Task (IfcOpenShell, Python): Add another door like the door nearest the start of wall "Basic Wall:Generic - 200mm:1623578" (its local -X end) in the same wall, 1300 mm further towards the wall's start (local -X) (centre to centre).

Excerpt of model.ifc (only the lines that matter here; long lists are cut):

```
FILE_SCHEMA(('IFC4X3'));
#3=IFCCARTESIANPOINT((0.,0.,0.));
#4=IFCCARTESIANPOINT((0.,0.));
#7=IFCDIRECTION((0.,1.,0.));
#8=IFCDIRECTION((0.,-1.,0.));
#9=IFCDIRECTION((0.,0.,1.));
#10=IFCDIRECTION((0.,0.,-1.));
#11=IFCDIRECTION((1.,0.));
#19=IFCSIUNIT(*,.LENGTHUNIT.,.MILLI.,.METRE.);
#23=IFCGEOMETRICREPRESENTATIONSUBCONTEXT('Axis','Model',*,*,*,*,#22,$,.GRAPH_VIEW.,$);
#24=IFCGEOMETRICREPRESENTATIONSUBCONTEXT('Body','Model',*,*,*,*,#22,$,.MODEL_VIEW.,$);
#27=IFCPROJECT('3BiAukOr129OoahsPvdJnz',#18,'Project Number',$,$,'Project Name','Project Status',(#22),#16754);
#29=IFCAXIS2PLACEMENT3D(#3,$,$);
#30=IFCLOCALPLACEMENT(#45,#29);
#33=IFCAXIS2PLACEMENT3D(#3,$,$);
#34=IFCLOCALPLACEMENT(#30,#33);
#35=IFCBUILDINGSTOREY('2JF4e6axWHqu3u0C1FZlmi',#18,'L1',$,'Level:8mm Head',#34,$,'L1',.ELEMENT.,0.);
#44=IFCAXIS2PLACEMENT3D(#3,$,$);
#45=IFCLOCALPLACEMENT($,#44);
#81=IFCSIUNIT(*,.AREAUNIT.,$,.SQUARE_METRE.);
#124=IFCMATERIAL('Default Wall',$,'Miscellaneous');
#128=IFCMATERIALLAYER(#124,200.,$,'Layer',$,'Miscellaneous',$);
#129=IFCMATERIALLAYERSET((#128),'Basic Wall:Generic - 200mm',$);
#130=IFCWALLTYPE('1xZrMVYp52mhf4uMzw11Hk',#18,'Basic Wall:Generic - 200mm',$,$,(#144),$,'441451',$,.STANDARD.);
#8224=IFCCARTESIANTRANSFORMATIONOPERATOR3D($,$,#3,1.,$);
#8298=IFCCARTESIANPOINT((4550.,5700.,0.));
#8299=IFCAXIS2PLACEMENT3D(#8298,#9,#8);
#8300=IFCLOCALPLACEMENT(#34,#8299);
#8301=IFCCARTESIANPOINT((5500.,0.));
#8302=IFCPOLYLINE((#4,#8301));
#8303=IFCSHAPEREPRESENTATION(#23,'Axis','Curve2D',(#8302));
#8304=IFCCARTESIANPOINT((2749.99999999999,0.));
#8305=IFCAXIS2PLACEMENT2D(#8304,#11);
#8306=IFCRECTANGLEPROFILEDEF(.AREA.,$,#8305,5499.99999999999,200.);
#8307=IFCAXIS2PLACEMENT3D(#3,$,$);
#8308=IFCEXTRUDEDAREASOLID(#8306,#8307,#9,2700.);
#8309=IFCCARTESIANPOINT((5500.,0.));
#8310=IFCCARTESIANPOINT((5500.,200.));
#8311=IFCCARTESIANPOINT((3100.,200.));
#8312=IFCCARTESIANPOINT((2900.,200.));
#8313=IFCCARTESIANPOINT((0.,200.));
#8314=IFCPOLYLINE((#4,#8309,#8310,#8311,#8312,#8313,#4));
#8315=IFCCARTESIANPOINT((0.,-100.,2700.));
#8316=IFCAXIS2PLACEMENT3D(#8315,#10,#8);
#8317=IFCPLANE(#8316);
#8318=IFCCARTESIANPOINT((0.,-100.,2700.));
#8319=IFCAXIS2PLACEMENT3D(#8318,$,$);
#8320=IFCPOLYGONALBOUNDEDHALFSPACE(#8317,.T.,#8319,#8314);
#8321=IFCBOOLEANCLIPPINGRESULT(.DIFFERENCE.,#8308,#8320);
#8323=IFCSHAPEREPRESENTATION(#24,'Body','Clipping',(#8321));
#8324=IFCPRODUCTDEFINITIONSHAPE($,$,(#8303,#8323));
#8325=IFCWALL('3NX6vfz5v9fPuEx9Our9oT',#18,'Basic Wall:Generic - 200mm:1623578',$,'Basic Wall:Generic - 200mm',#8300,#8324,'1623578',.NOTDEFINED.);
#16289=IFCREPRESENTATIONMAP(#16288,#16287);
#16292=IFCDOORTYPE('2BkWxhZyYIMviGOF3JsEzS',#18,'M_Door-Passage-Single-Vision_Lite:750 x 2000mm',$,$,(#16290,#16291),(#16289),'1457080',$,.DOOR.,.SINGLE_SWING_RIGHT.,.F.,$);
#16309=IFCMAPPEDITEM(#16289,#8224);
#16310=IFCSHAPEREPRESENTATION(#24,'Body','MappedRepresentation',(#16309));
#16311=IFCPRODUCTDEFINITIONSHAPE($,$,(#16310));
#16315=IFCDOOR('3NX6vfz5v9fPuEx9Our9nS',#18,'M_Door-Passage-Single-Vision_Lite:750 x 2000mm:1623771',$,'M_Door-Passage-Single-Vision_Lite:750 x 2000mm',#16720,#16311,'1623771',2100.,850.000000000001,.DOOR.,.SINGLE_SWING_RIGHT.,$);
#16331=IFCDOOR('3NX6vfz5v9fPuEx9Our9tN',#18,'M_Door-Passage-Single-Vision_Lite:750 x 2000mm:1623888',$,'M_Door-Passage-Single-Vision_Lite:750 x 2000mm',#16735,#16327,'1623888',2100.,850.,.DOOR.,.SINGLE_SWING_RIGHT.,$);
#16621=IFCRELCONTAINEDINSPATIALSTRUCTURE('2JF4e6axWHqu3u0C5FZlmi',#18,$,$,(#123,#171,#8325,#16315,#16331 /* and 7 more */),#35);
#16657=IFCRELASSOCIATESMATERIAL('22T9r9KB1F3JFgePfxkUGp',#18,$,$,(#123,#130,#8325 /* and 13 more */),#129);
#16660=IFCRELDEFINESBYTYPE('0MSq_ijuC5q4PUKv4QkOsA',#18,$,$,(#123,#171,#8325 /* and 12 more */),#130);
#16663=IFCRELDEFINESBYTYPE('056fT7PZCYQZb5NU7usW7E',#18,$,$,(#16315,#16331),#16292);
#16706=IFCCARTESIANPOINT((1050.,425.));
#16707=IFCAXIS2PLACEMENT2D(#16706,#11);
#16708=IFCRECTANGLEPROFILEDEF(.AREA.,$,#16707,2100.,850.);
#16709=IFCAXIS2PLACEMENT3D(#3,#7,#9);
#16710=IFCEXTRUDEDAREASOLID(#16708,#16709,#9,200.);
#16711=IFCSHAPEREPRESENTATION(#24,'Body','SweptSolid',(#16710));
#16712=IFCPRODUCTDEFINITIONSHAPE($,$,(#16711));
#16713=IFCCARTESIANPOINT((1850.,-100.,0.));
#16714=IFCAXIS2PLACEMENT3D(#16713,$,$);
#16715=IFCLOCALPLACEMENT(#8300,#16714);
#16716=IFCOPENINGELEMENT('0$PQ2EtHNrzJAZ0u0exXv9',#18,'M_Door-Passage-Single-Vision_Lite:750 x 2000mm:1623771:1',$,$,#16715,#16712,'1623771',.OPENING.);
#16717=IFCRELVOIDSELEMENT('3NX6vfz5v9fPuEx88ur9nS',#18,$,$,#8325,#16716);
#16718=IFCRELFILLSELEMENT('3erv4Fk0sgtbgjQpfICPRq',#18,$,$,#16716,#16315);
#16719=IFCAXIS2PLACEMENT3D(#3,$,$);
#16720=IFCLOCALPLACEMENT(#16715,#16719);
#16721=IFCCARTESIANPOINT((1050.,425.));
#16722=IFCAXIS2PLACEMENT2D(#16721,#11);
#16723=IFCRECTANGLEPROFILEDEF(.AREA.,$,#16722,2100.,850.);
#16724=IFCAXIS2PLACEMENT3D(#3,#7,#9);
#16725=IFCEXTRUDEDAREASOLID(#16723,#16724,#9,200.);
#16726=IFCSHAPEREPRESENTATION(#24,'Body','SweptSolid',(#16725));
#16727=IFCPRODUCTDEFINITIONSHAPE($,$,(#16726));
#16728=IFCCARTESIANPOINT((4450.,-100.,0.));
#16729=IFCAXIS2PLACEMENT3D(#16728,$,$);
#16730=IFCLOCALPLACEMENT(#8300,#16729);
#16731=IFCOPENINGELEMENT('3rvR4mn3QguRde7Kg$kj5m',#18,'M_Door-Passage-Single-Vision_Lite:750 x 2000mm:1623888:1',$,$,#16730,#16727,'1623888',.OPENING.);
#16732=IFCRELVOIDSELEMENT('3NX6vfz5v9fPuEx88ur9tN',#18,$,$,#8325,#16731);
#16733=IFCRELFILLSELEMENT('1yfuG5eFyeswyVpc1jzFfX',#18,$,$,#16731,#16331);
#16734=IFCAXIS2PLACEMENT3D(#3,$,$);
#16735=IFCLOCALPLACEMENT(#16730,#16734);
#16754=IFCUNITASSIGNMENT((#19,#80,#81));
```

```python
import ifcopenshell
import ifcopenshell.api.feature
import ifcopenshell.api.geometry
import ifcopenshell.api.root
import ifcopenshell.geom
import ifcopenshell.util.element
import ifcopenshell.util.placement
import ifcopenshell.util.shape
import ifcopenshell.util.unit

model = ifcopenshell.open("model.ifc")
unit_scale = ifcopenshell.util.unit.calculate_unit_scale(model)
settings = ifcopenshell.geom.settings()


def volume(element):
    """Net volume in cubic metres, openings subtracted."""
    shape = ifcopenshell.geom.create_shape(settings, element)
    return ifcopenshell.util.shape.get_volume(shape.geometry)


def reuse_history(source, copy):
    """copy_class also copies each property set's owner history, people and application; keep the originals."""
    for rel in copy.IsDefinedBy:
        if rel.is_a("IfcRelDefinesByProperties") and (history := rel.RelatingPropertyDefinition.OwnerHistory):
            rel.RelatingPropertyDefinition.OwnerHistory = source.OwnerHistory
            ifcopenshell.util.element.remove_deep2(model, history)


door = model.by_id(16315)
opening = door.FillsVoids[0].RelatingOpeningElement
wall = opening.VoidsElements[0].RelatingBuildingElement
before = volume(wall)
shift = ifcopenshell.util.placement.get_local_placement(wall.ObjectPlacement)[:3, 0] * -1.3 / unit_scale

# copy_class copies the void relationship, type, container and properties, but no geometry.
new_opening = ifcopenshell.api.root.copy_class(model, product=opening)
new_opening.Representation = ifcopenshell.util.element.copy_deep(
    model, opening.Representation, exclude=["IfcGeometricRepresentationContext", "IfcRepresentationMap"]
)
new_opening.Name = "M_Door-Passage-Single-Vision_Lite:750 x 2000mm"
new_opening.Tag = None
new_door = ifcopenshell.api.root.copy_class(model, product=door)
new_door.Representation = ifcopenshell.util.element.copy_deep(
    model, door.Representation, exclude=["IfcGeometricRepresentationContext", "IfcRepresentationMap"]
)
new_door.Name = "M_Door-Passage-Single-Vision_Lite:750 x 2000mm"
new_door.Tag = None
reuse_history(door, new_door)
ifcopenshell.api.feature.add_filling(model, opening=new_opening, element=new_door)

for old, new in ((opening, new_opening), (door, new_door)):
    matrix = ifcopenshell.util.placement.get_local_placement(old.ObjectPlacement)
    matrix[:3, 3] += shift
    ifcopenshell.api.geometry.edit_object_placement(model, product=new, matrix=matrix, is_si=False)

after = volume(wall)

print(f"wall volume {before:.3f} -> {after:.3f} m3")

model.write("model_updated.ifc")
```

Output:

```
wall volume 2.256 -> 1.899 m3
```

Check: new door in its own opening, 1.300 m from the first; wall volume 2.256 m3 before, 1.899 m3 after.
